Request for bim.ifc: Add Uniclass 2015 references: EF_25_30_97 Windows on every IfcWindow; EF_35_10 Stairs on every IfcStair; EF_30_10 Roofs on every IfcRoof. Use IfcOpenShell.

First a look at what the model holds.

```python
import ifcopenshell

model = ifcopenshell.open("bim.ifc")
print(model.schema)
print("classifications:", [c.Name for c in model.by_type("IfcClassification")])
for ifc_class in ("IfcDoor", "IfcRoof", "IfcStair", "IfcWall", "IfcWindow"):
    print(ifc_class, len(model.by_type(ifc_class)))
```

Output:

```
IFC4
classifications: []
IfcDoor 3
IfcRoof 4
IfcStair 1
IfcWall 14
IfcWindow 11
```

```python
import ifcopenshell
import ifcopenshell.api.classification

model = ifcopenshell.open("bim.ifc")

system = ifcopenshell.api.classification.add_classification(model, classification="Uniclass 2015")

codes = {
    "IfcWindow": ("EF_25_30_97", "Windows"),
    "IfcStair": ("EF_35_10", "Stairs"),
    "IfcRoof": ("EF_30_10", "Roofs"),
}
for ifc_class, (code, name) in codes.items():
    products = model.by_type(ifc_class)
    ifcopenshell.api.classification.add_reference(
        model, products=products, classification=system, identification=code, name=name
    )
    print(code, len(products))

model.write("bim_rev.ifc")
```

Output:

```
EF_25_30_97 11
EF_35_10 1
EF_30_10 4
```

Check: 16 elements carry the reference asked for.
